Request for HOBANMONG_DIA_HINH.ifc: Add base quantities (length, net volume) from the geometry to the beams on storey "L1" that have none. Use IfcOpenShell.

First a look at what the model holds.

```python
import ifcopenshell
import ifcopenshell.util.element
import ifcopenshell.util.unit

model = ifcopenshell.open("HOBANMONG_DIA_HINH.ifc")
print(model.schema)
for unit_type in ("LENGTHUNIT", "AREAUNIT", "VOLUMEUNIT"):
    print(unit_type, ifcopenshell.util.unit.calculate_unit_scale(model, unit_type))
storey = next(s for s in model.by_type("IfcBuildingStorey") if s.Name == "L1")
beams = [e for e in ifcopenshell.util.element.get_decomposition(storey) if e.is_a("IfcBeam")]
for e in sorted(beams, key=lambda e: e.id()):
    print(e.id(), e.is_a(), e.Name, list(ifcopenshell.util.element.get_psets(e, qtos_only=True)), sep=" | ")
```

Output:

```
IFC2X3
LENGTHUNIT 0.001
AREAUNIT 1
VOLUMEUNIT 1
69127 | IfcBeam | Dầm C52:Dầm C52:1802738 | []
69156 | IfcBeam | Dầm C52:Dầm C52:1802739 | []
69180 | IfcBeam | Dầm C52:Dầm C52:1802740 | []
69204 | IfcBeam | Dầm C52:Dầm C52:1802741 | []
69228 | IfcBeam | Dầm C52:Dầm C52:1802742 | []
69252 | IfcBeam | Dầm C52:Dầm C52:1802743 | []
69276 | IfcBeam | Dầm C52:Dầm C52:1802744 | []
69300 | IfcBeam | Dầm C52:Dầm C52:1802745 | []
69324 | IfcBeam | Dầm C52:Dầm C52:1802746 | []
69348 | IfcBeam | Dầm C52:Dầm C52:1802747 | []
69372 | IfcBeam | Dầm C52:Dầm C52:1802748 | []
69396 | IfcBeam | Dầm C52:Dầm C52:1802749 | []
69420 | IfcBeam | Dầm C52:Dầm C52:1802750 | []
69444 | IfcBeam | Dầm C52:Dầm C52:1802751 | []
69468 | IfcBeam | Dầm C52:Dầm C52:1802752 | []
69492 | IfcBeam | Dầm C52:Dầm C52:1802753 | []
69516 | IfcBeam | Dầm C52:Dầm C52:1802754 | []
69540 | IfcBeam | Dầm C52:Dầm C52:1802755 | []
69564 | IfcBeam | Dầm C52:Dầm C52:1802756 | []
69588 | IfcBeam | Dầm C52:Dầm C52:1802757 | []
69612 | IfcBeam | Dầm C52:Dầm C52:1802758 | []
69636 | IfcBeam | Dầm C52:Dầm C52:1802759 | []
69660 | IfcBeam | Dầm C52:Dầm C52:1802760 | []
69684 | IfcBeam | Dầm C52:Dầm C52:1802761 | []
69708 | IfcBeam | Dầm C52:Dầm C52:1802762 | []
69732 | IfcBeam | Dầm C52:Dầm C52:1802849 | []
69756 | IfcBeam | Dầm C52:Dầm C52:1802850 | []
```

```python
import ifcopenshell
import ifcopenshell.api.pset
import ifcopenshell.geom
import ifcopenshell.util.element
import ifcopenshell.util.shape
import ifcopenshell.util.unit

model = ifcopenshell.open("HOBANMONG_DIA_HINH.ifc")
unit_scale = ifcopenshell.util.unit.calculate_unit_scale(model)
volume_scale = ifcopenshell.util.unit.calculate_unit_scale(model, "VOLUMEUNIT")
settings = ifcopenshell.geom.settings()

storey = next(s for s in model.by_type("IfcBuildingStorey") if s.Name == "L1")
beams = [e for e in ifcopenshell.util.element.get_decomposition(storey) if e.is_a("IfcBeam")]

for e in sorted(beams, key=lambda e: e.id()):
    if ifcopenshell.util.element.get_psets(e, qtos_only=True, should_inherit=False):
        continue
    # Geometry comes back in metres, in the element's own axes.
    shape = ifcopenshell.geom.create_shape(settings, e)
    values = {
        "Length": ifcopenshell.util.shape.get_max_xyz(shape.geometry) / unit_scale,
        "NetVolume": ifcopenshell.util.shape.get_volume(shape.geometry) / volume_scale,
    }
    qto = ifcopenshell.api.pset.add_qto(model, product=e, name="BaseQuantities")
    ifcopenshell.api.pset.edit_qto(model, qto=qto, properties=values)
    print(e.id(), {k: round(v, 3) for k, v in values.items()})

model.write("HOBANMONG_DIA_HINH_edited.ifc")
```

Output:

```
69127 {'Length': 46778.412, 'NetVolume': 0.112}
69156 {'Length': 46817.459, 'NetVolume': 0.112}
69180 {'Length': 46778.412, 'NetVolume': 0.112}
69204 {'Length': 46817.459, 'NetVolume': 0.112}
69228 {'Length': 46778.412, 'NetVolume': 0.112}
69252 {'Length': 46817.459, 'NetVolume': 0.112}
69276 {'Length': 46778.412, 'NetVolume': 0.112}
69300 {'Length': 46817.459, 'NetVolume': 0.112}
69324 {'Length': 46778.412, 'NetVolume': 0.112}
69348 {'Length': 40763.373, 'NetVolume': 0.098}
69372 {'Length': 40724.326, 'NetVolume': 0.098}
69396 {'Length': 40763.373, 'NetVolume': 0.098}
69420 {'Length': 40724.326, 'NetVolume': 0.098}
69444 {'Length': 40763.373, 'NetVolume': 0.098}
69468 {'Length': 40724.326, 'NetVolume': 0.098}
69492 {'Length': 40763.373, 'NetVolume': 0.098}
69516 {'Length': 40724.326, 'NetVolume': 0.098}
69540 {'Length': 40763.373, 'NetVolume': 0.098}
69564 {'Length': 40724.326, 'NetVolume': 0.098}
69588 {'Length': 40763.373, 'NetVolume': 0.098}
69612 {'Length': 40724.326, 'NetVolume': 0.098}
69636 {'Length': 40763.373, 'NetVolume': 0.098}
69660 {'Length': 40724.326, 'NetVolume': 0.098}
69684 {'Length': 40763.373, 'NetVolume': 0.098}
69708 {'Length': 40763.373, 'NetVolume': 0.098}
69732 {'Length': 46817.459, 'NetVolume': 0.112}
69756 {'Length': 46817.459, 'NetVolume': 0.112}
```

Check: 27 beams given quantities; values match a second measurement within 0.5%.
